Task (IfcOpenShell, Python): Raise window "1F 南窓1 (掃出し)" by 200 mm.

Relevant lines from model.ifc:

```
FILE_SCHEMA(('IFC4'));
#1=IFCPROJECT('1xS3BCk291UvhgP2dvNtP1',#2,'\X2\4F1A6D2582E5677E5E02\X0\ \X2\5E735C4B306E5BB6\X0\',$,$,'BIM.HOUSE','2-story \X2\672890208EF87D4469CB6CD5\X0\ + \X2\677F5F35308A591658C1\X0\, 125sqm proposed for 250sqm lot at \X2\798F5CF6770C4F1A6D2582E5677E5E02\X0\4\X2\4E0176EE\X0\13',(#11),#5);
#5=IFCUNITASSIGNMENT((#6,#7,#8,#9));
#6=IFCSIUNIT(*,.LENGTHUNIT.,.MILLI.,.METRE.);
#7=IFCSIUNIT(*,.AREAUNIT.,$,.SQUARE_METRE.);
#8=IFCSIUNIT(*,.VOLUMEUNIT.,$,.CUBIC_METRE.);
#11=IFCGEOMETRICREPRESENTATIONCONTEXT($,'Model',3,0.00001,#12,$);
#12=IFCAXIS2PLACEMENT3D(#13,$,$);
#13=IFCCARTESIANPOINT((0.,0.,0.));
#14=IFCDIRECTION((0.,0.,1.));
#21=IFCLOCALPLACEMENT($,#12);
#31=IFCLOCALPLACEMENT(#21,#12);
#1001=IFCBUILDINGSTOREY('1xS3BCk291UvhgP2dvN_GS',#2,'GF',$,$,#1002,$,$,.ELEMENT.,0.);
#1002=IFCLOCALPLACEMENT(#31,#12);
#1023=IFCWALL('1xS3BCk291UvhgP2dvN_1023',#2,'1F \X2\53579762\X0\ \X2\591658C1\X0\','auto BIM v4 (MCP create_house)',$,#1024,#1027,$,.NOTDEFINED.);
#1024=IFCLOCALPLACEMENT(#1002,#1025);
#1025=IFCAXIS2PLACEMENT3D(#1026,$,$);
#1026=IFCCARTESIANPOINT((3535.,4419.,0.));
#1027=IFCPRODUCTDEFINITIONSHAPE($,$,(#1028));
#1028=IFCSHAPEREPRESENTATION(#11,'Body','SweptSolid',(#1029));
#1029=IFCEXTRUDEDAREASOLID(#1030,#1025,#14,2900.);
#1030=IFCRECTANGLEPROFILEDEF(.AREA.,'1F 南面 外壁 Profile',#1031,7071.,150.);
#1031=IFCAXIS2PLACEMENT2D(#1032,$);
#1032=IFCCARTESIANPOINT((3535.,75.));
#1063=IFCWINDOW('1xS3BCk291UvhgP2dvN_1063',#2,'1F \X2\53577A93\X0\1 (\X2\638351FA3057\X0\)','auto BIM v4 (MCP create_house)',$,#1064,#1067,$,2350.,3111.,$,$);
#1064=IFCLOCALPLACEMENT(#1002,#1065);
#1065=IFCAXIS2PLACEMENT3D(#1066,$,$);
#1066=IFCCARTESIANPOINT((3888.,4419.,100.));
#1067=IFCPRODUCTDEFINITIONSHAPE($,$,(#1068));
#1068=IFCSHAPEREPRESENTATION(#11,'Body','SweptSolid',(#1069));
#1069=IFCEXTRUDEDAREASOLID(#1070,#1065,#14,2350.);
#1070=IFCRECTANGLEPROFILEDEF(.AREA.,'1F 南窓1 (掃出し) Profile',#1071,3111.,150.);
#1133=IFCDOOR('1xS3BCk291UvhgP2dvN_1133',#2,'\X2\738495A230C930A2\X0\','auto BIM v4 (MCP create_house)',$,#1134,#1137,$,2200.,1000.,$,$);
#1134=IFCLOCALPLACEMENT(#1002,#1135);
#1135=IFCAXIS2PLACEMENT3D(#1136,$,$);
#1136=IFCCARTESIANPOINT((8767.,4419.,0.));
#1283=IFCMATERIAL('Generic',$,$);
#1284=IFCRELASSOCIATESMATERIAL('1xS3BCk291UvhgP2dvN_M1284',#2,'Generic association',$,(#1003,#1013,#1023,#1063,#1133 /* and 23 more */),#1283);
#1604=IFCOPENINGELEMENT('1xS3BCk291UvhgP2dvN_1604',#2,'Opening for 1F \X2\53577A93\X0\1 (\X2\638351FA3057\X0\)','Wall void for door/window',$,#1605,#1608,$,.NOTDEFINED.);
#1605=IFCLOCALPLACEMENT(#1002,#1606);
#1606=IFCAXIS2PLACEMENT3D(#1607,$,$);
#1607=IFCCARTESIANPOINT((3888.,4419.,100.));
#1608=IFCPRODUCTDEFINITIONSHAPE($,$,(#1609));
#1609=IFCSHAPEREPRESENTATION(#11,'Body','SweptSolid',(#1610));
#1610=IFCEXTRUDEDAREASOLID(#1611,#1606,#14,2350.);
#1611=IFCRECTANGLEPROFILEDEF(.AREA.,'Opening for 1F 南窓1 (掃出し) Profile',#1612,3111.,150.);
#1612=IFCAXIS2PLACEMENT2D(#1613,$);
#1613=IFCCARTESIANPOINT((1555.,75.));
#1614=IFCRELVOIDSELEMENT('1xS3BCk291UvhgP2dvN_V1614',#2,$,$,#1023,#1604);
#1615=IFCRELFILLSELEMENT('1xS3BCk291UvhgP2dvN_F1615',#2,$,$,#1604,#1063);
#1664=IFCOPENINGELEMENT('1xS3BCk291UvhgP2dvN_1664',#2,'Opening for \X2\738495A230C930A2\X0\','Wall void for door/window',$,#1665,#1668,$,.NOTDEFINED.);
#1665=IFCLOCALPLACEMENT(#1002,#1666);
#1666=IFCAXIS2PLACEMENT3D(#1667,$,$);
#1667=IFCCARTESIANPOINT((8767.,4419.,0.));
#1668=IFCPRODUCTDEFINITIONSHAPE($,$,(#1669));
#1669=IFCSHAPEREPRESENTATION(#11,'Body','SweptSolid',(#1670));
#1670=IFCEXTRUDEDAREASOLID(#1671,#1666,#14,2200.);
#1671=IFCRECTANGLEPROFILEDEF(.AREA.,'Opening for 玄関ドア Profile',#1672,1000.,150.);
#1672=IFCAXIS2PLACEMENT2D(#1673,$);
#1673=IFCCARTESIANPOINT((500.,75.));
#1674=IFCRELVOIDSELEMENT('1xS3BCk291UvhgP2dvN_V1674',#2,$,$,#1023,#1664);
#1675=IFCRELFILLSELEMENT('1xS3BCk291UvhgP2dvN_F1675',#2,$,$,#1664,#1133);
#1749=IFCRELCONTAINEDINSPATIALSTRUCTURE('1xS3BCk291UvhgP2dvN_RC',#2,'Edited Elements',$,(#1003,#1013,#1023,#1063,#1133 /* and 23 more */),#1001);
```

```python
import numpy as np
import ifcopenshell
import ifcopenshell.api.geometry
import ifcopenshell.util.placement
import ifcopenshell.util.unit

model = ifcopenshell.open("model.ifc")
unit_scale = ifcopenshell.util.unit.calculate_unit_scale(model)

window = model.by_guid("1xS3BCk291UvhgP2dvN_1063")
opening = window.FillsVoids[0].RelatingOpeningElement
dz = 0.2 / unit_scale

shift = np.array([0.0, 0.0, dz])
# The window is not placed relative to its opening, so move both.
for product in (opening, window):
    matrix = ifcopenshell.util.placement.get_local_placement(product.ObjectPlacement)
    matrix[:3, 3] += shift
    ifcopenshell.api.geometry.edit_object_placement(model, product=product, matrix=matrix, is_si=False)

print(f"moved by {dz * unit_scale:+.3f} m")

model.write("model_rev.ifc")
```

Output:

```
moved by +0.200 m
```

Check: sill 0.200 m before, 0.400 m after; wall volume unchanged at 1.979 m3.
